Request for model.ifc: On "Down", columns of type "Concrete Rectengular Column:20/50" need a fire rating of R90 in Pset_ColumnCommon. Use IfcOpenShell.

First a look at what the model holds.

```python
import ifcopenshell
import ifcopenshell.util.element

model = ifcopenshell.open("model.ifc")
print(model.schema)
storey = next(s for s in model.by_type("IfcBuildingStorey") if s.Name == "Down")
columns = [e for e in ifcopenshell.util.element.get_decomposition(storey) if e.is_a("IfcColumn")]
seen = {}
for e in columns:
    element_type = ifcopenshell.util.element.get_type(e)
    key = (element_type.Name if element_type != e and element_type else None, ifcopenshell.util.element.get_pset(e, "Pset_ColumnCommon", "FireRating"))
    seen[key] = seen.get(key, 0) + 1
for (name, value), count in sorted(seen.items(), key=str):
    print(count, "x", name, "|", value)
```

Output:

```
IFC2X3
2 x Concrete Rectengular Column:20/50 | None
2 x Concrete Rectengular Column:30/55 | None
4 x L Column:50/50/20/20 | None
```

```python
import ifcopenshell
import ifcopenshell.api.pset
import ifcopenshell.util.element

model = ifcopenshell.open("model.ifc")

storey = next(s for s in model.by_type("IfcBuildingStorey") if s.Name == "Down")
columns = [e for e in ifcopenshell.util.element.get_decomposition(storey) if e.is_a("IfcColumn")]

count = 0
for e in columns:
    element_type = ifcopenshell.util.element.get_type(e)
    if element_type in (None, e) or element_type.Name != "Concrete Rectengular Column:20/50":
        continue
    # add_pset returns the element's existing set when there is one.
    pset = ifcopenshell.api.pset.add_pset(model, product=e, name="Pset_ColumnCommon")
    ifcopenshell.api.pset.edit_pset(model, pset=pset, properties={"FireRating": "R90"})
    count += 1

print(count, "columns updated")

model.write("model_updated.ifc")
```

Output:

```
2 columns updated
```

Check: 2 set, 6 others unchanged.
